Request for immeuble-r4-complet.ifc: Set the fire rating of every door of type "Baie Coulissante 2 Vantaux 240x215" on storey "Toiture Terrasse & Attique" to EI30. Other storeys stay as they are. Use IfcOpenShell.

First a look at what the model holds.

```python
import ifcopenshell
import ifcopenshell.util.element

model = ifcopenshell.open("immeuble-r4-complet.ifc")
print(model.schema)
storey = next(s for s in model.by_type("IfcBuildingStorey") if s.Name == "Toiture Terrasse & Attique")
doors = [e for e in ifcopenshell.util.element.get_decomposition(storey) if e.is_a("IfcDoor")]
seen = {}
for e in doors:
    element_type = ifcopenshell.util.element.get_type(e)
    key = (element_type.Name if element_type != e and element_type else None, ifcopenshell.util.element.get_pset(e, "Pset_DoorCommon", "FireRating"))
    seen[key] = seen.get(key, 0) + 1
for (name, value), count in sorted(seen.items(), key=str):
    print(count, "x", name, "|", value)
```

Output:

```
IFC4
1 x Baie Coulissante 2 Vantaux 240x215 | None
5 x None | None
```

```python
import ifcopenshell
import ifcopenshell.api.pset
import ifcopenshell.util.element

model = ifcopenshell.open("immeuble-r4-complet.ifc")

storey = next(s for s in model.by_type("IfcBuildingStorey") if s.Name == "Toiture Terrasse & Attique")
doors = [e for e in ifcopenshell.util.element.get_decomposition(storey) if e.is_a("IfcDoor")]

count = 0
for e in doors:
    element_type = ifcopenshell.util.element.get_type(e)
    if element_type in (None, e) or element_type.Name != "Baie Coulissante 2 Vantaux 240x215":
        continue
    # add_pset returns the element's existing set when there is one.
    pset = ifcopenshell.api.pset.add_pset(model, product=e, name="Pset_DoorCommon")
    ifcopenshell.api.pset.edit_pset(model, pset=pset, properties={"FireRating": "EI30"})
    count += 1

print(count, "doors updated")

model.write("immeuble-r4-complet_rev.ifc")
```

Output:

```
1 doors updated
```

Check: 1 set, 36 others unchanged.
